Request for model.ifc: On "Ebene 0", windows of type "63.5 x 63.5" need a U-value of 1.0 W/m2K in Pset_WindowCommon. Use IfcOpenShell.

First a look at what the model holds.

```python
import ifcopenshell
import ifcopenshell.util.element

model = ifcopenshell.open("model.ifc")
print(model.schema)
storey = next(s for s in model.by_type("IfcBuildingStorey") if s.Name == "Ebene 0")
windows = [e for e in ifcopenshell.util.element.get_decomposition(storey) if e.is_a("IfcWindow")]
seen = {}
for e in windows:
    element_type = ifcopenshell.util.element.get_type(e)
    key = (element_type.Name if element_type != e and element_type else None, ifcopenshell.util.element.get_pset(e, "Pset_WindowCommon", "ThermalTransmittance"))
    seen[key] = seen.get(key, 0) + 1
for (name, value), count in sorted(seen.items(), key=str):
    print(count, "x", name, "|", value)
```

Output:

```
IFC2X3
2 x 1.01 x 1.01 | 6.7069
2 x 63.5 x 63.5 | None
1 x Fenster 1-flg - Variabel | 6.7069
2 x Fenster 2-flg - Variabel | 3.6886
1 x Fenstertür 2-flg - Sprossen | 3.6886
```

```python
import ifcopenshell
import ifcopenshell.api.pset
import ifcopenshell.util.element

model = ifcopenshell.open("model.ifc")

storey = next(s for s in model.by_type("IfcBuildingStorey") if s.Name == "Ebene 0")
windows = [e for e in ifcopenshell.util.element.get_decomposition(storey) if e.is_a("IfcWindow")]

count = 0
for e in windows:
    element_type = ifcopenshell.util.element.get_type(e)
    if element_type in (None, e) or element_type.Name != "63.5 x 63.5":
        continue
    # add_pset returns the element's existing set when there is one.
    pset = ifcopenshell.api.pset.add_pset(model, product=e, name="Pset_WindowCommon")
    ifcopenshell.api.pset.edit_pset(model, pset=pset, properties={"ThermalTransmittance": 1.0})
    count += 1

print(count, "windows updated")

model.write("model_updated.ifc")
```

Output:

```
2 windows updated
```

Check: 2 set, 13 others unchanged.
